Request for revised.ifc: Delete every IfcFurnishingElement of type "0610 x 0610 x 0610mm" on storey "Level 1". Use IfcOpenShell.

First a look at what the model holds.

```python
import ifcopenshell
import ifcopenshell.util.element

model = ifcopenshell.open("revised.ifc")
print(model.schema)
storey = next(s for s in model.by_type("IfcBuildingStorey") if s.Name == "Level 1")
furniture = [e for e in ifcopenshell.util.element.get_decomposition(storey) if e.is_a("IfcFurnishingElement")]
seen = {}
for e in furniture:
    element_type = ifcopenshell.util.element.get_type(e)
    name = element_type.Name if element_type not in (None, e) else None
    seen[name] = seen.get(name, 0) + 1
for name, count in sorted(seen.items(), key=str):
    print(count, "x", name)
```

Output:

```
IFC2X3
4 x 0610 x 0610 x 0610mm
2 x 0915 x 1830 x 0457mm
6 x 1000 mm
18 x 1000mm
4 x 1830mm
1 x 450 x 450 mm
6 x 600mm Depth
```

```python
import ifcopenshell
import ifcopenshell.api.root
import ifcopenshell.util.element

model = ifcopenshell.open("revised.ifc")

storey = next(s for s in model.by_type("IfcBuildingStorey") if s.Name == "Level 1")
furniture = [e for e in ifcopenshell.util.element.get_decomposition(storey) if e.is_a("IfcFurnishingElement")]
targets = [e for e in furniture if (t := ifcopenshell.util.element.get_type(e)) not in (None, e) and t.Name == "0610 x 0610 x 0610mm"]

for e in targets:
    ifcopenshell.api.root.remove_product(model, product=e)
print(len(targets), "removed")

model.write("revised-out.ifc")
```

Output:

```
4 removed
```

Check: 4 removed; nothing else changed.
